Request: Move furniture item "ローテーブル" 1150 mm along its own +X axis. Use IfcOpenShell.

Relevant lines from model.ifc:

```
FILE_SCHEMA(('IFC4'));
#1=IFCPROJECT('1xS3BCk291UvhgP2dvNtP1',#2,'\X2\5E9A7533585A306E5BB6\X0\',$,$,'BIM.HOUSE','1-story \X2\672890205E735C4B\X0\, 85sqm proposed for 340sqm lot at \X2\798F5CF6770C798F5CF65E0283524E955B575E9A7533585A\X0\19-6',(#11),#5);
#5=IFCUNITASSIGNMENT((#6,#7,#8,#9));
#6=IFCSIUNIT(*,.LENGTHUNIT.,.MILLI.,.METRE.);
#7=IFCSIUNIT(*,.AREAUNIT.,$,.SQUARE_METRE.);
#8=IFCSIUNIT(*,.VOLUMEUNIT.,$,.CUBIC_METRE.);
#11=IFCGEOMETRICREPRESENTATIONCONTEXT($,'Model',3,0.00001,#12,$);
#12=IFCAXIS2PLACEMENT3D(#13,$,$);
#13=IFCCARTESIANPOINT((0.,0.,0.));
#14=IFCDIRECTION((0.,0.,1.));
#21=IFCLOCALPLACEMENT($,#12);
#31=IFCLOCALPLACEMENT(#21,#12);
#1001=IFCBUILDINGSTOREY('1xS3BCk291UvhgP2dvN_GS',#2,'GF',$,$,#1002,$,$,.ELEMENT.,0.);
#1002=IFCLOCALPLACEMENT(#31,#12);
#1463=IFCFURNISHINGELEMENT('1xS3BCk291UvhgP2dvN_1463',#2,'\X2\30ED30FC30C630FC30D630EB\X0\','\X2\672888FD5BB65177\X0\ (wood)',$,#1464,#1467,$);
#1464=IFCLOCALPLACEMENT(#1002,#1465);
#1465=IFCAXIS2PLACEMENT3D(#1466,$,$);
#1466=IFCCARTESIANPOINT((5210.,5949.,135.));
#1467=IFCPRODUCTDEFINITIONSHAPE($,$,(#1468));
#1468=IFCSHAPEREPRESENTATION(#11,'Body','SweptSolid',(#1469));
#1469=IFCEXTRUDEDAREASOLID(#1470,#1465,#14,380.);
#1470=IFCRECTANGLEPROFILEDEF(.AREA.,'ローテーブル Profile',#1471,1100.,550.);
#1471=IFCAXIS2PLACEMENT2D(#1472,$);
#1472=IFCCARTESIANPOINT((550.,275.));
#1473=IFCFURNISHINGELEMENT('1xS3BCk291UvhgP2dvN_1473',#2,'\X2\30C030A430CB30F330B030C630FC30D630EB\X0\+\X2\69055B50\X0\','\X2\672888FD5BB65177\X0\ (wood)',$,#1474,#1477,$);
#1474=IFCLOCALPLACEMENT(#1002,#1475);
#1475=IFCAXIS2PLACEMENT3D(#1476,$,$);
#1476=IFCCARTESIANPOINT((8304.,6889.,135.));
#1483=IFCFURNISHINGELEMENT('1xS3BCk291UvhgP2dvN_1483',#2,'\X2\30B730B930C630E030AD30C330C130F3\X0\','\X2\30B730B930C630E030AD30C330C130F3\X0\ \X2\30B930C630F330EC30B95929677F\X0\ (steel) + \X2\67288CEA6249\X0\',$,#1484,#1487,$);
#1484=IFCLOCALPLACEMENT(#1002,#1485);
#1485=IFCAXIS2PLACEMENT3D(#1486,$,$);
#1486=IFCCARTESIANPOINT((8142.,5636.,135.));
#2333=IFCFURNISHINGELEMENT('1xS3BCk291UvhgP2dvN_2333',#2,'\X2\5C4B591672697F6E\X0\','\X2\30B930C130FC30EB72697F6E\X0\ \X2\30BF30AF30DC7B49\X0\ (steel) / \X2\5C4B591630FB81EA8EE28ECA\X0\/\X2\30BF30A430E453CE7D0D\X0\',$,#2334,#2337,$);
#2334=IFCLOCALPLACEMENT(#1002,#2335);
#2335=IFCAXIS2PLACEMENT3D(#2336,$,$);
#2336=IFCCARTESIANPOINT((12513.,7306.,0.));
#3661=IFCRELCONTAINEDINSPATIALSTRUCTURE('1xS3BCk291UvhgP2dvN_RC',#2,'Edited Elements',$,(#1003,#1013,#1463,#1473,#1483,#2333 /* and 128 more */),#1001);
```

```python
import ifcopenshell
import ifcopenshell.api.geometry
import ifcopenshell.util.placement
import ifcopenshell.util.unit

model = ifcopenshell.open("model.ifc")
unit_scale = ifcopenshell.util.unit.calculate_unit_scale(model)

item = model.by_id(1463)
matrix = ifcopenshell.util.placement.get_local_placement(item.ObjectPlacement)
matrix[:3, 3] += matrix[:3, 0] * 1.15 / unit_scale
ifcopenshell.api.geometry.edit_object_placement(model, product=item, matrix=matrix, is_si=False)

print(ifcopenshell.util.placement.get_local_placement(item.ObjectPlacement).round(3) + 0.0)

model.write("model_edited.ifc")
```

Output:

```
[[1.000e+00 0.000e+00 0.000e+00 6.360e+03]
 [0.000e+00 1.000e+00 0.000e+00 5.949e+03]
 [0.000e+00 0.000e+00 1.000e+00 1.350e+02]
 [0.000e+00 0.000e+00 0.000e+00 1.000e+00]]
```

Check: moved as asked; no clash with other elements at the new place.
